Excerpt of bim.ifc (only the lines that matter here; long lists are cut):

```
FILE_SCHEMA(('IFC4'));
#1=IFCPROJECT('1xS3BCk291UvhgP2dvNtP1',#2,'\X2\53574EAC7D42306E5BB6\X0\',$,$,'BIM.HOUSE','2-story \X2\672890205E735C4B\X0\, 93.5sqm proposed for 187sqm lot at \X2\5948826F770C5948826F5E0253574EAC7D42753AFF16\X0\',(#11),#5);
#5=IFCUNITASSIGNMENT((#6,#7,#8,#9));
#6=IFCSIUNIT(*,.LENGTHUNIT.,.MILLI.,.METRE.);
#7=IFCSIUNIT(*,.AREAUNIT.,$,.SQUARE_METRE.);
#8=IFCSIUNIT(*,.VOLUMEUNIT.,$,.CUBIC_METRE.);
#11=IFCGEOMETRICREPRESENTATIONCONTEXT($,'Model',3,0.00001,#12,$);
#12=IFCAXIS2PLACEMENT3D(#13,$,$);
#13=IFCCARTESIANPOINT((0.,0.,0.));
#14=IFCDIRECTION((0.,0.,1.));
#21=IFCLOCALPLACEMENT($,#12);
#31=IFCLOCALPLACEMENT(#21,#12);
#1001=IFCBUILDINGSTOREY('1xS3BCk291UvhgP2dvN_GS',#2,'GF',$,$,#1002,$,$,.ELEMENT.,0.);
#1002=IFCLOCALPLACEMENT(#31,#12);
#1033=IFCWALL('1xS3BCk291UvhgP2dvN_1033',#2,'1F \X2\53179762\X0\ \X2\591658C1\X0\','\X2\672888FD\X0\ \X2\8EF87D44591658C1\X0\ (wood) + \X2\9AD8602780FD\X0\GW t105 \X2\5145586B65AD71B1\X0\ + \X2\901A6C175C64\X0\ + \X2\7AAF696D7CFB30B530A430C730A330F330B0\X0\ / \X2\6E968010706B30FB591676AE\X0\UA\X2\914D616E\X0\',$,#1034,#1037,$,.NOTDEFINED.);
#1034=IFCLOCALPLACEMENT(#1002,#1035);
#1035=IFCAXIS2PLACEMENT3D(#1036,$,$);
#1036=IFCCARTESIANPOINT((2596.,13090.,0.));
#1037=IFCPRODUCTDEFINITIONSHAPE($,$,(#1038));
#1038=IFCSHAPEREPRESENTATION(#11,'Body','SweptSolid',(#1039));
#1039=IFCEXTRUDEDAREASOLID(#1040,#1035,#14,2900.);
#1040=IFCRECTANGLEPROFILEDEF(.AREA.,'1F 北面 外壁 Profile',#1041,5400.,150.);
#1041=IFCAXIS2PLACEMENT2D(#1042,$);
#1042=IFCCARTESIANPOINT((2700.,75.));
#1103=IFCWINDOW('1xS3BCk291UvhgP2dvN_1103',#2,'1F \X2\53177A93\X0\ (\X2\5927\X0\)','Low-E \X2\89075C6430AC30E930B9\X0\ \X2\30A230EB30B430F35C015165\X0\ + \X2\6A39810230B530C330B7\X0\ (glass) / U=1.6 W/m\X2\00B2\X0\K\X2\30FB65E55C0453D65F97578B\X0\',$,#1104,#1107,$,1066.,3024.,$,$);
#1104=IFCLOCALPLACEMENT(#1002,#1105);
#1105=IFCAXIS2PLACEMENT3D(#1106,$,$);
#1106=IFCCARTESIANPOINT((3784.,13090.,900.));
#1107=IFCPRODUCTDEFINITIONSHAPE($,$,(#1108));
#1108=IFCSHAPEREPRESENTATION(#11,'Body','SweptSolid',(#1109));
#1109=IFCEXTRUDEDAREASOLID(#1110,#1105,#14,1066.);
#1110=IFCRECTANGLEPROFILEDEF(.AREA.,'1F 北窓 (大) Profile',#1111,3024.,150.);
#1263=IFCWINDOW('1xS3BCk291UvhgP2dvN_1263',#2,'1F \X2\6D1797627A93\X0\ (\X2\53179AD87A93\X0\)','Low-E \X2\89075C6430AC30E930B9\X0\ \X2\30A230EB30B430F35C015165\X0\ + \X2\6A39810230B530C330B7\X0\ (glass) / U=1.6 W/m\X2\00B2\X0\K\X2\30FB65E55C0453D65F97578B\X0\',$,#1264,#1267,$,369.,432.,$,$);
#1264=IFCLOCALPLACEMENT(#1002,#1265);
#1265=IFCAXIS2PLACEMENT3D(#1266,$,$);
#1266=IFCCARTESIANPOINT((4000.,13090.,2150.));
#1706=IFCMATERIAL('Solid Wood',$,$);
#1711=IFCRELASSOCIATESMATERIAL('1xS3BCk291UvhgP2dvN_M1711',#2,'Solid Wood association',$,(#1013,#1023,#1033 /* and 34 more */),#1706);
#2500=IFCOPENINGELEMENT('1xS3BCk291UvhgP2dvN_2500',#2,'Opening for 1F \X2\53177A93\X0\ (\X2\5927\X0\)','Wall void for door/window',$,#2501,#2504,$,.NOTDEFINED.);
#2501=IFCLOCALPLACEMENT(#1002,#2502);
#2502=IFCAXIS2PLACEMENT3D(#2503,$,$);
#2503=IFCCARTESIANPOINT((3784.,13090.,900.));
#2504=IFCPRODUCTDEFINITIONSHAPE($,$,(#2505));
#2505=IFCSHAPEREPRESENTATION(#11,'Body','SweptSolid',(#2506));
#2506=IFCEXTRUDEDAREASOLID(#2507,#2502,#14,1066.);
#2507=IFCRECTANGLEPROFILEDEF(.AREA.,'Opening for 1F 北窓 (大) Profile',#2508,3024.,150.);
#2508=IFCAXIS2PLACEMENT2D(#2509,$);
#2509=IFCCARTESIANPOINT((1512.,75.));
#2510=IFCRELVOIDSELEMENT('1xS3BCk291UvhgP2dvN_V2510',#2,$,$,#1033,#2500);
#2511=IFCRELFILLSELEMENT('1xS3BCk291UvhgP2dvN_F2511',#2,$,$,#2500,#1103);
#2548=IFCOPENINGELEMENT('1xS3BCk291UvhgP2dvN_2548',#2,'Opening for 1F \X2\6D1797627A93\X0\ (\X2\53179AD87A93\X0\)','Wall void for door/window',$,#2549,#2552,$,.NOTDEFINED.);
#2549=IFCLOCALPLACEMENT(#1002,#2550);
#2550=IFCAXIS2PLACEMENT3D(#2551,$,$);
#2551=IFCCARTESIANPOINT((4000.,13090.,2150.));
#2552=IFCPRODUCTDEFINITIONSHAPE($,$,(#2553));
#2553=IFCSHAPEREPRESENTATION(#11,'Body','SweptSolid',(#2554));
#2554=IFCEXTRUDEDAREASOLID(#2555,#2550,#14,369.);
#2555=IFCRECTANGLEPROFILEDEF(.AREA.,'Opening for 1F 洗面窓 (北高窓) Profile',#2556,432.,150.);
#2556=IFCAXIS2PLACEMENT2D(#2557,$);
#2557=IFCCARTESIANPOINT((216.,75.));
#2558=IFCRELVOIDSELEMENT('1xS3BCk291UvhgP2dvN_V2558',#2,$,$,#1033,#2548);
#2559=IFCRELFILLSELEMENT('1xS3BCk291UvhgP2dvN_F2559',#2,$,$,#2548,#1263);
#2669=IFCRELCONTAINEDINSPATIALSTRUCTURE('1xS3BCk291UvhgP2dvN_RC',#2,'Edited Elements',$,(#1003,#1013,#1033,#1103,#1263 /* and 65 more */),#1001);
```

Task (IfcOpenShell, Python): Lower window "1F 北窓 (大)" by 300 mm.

```python
import numpy as np
import ifcopenshell
import ifcopenshell.api.geometry
import ifcopenshell.util.placement
import ifcopenshell.util.unit

model = ifcopenshell.open("bim.ifc")
unit_scale = ifcopenshell.util.unit.calculate_unit_scale(model)

window = model.by_guid("1xS3BCk291UvhgP2dvN_1103")
opening = window.FillsVoids[0].RelatingOpeningElement
dz = -0.3 / unit_scale

shift = np.array([0.0, 0.0, dz])
# The window is not placed relative to its opening, so move both.
for product in (opening, window):
    matrix = ifcopenshell.util.placement.get_local_placement(product.ObjectPlacement)
    matrix[:3, 3] += shift
    ifcopenshell.api.geometry.edit_object_placement(model, product=product, matrix=matrix, is_si=False)

print(f"moved by {dz * unit_scale:+.3f} m")

model.write("bim-out.ifc")
```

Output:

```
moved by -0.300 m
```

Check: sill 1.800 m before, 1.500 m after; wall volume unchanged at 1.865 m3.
